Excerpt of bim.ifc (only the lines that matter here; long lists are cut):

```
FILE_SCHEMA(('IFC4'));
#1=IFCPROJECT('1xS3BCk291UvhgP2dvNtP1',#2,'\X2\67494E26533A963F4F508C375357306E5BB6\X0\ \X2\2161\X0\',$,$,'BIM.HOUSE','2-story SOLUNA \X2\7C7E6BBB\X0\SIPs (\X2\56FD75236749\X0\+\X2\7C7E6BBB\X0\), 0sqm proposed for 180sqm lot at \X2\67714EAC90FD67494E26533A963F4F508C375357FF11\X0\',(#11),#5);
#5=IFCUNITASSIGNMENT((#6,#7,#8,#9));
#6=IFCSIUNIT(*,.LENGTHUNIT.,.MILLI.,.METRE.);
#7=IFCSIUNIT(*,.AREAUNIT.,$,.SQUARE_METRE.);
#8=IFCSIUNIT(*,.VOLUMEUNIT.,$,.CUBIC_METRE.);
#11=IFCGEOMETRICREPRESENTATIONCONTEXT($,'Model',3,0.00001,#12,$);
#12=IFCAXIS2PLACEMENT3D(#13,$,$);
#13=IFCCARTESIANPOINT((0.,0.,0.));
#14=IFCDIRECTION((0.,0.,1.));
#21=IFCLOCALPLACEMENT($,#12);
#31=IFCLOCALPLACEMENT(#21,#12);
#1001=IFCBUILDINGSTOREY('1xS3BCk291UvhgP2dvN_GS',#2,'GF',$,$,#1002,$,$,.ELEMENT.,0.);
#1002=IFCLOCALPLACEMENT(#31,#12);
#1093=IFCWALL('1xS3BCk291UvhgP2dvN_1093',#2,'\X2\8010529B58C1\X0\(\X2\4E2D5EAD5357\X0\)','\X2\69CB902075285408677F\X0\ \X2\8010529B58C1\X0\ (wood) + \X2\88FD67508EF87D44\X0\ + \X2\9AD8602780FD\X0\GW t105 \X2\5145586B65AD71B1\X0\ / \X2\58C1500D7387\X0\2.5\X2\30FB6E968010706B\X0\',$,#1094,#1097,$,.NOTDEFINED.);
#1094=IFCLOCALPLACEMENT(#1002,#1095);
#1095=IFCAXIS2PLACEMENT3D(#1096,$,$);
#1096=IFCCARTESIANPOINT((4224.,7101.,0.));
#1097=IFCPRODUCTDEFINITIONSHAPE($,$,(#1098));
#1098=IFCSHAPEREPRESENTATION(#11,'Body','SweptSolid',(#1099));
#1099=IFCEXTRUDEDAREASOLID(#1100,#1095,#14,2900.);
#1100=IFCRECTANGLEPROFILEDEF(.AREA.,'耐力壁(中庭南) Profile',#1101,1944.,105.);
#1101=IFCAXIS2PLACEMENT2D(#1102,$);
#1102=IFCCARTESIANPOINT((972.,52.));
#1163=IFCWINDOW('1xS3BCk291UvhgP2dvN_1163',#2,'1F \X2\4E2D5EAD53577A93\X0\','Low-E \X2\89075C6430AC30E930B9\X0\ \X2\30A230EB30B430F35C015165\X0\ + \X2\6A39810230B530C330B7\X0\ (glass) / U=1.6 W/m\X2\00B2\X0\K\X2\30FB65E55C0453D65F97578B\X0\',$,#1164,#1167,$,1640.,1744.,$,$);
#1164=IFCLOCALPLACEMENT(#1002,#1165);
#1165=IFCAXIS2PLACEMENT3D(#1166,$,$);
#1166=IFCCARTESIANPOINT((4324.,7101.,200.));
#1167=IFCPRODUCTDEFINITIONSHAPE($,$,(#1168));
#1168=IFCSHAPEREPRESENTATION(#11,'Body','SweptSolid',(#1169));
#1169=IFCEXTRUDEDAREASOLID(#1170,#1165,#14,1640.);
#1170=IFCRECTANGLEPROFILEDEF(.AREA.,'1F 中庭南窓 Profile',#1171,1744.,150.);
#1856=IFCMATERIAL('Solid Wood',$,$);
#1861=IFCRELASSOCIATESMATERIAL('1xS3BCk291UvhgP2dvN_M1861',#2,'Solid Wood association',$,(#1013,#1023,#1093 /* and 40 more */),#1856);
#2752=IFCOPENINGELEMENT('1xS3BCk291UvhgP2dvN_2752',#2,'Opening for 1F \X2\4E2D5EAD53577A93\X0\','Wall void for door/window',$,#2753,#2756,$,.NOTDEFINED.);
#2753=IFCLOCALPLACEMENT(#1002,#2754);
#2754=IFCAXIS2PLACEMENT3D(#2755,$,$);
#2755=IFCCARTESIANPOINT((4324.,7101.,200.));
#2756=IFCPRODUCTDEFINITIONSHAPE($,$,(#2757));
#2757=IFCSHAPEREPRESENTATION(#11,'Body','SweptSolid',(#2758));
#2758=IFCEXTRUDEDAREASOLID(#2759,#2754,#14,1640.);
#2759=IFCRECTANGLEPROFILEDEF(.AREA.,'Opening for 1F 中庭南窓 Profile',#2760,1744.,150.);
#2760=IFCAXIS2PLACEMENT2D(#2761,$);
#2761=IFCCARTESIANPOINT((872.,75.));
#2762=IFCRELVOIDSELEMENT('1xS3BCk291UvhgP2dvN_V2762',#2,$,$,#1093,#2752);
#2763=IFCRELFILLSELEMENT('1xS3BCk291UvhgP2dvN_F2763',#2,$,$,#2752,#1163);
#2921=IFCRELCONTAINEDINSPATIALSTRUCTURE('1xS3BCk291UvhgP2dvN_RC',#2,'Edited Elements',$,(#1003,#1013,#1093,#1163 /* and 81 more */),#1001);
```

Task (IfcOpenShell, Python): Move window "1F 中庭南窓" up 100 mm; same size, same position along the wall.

```python
import numpy as np
import ifcopenshell
import ifcopenshell.api.geometry
import ifcopenshell.util.placement
import ifcopenshell.util.unit

model = ifcopenshell.open("bim.ifc")
unit_scale = ifcopenshell.util.unit.calculate_unit_scale(model)

window = model.by_guid("1xS3BCk291UvhgP2dvN_1163")
opening = window.FillsVoids[0].RelatingOpeningElement
dz = 100.0

shift = np.array([0.0, 0.0, dz])
# The window is not placed relative to its opening, so move both.
for product in (opening, window):
    matrix = ifcopenshell.util.placement.get_local_placement(product.ObjectPlacement)
    matrix[:3, 3] += shift
    ifcopenshell.api.geometry.edit_object_placement(model, product=product, matrix=matrix, is_si=False)

print(f"moved by {dz * unit_scale:+.3f} m")

model.write("bim_rev.ifc")
```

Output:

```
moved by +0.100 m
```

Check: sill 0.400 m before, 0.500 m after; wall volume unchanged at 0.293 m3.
